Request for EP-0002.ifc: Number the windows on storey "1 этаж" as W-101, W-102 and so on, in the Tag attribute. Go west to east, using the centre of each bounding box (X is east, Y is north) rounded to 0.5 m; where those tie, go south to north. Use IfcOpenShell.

First a look at what the model holds.

```python
import ifcopenshell
import ifcopenshell.util.element
import ifcopenshell.util.placement

model = ifcopenshell.open("EP-0002.ifc")
print(model.schema)
storey = next(s for s in model.by_type("IfcBuildingStorey") if s.Name == "1 этаж")
windows = [e for e in ifcopenshell.util.element.get_decomposition(storey) if e.is_a("IfcWindow")]
for e in sorted(windows, key=lambda e: e.id()):
    origin = ifcopenshell.util.placement.get_local_placement(e.ObjectPlacement)[:3, 3]
    print(e.id(), e.Tag, e.Name, origin.round(2) + 0.0, sep=" | ")
```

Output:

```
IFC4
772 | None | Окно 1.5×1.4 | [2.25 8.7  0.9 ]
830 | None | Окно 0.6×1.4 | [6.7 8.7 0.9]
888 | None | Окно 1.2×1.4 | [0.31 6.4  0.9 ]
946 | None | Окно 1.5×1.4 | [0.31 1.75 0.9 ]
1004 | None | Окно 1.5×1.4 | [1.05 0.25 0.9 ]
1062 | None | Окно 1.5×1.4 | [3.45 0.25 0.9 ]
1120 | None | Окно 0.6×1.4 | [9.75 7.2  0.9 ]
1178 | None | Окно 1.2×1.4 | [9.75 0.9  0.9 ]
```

```python
import ifcopenshell
import ifcopenshell.geom
import ifcopenshell.util.element
import ifcopenshell.util.shape

model = ifcopenshell.open("EP-0002.ifc")
settings = ifcopenshell.geom.settings()
settings.set("use-world-coords", True)


def centre(element):
    shape = ifcopenshell.geom.create_shape(settings, element)
    return ifcopenshell.util.shape.get_bbox_centroid(shape.geometry)


storey = next(s for s in model.by_type("IfcBuildingStorey") if s.Name == "1 этаж")
windows = [e for e in ifcopenshell.util.element.get_decomposition(storey) if e.is_a("IfcWindow")]

# Insertion points can sit at a corner or the storey origin, so sort by the geometry (in metres).
centres = {e: centre(e) for e in windows}
windows.sort(key=lambda e: (round(centres[e][0] / 0.5), centres[e][1]))

for i, e in enumerate(windows, start=1):
    number = f"W-1{i:02d}"
    e.Tag = number
    print(e.id(), number)

model.write("EP-0002_edited.ifc")
```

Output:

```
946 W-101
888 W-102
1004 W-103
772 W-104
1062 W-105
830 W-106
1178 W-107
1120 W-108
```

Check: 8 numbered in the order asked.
